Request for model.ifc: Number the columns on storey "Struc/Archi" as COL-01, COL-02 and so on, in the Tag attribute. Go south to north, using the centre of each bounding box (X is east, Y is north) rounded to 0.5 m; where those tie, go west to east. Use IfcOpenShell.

First a look at what the model holds.

```python
import ifcopenshell
import ifcopenshell.util.element
import ifcopenshell.util.placement

model = ifcopenshell.open("model.ifc")
print(model.schema)
storey = next(s for s in model.by_type("IfcBuildingStorey") if s.Name == "Struc/Archi")
columns = [e for e in ifcopenshell.util.element.get_decomposition(storey) if e.is_a("IfcColumn")]
for e in sorted(columns, key=lambda e: e.id()):
    origin = ifcopenshell.util.placement.get_local_placement(e.ObjectPlacement)[:3, 3]
    print(e.id(), e.Tag, e.Name, origin.round(2) + 0.0, sep=" | ")
```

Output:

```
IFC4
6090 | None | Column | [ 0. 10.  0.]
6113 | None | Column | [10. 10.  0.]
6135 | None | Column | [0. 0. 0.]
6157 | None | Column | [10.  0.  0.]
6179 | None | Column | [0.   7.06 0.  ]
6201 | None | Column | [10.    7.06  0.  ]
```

```python
import ifcopenshell
import ifcopenshell.geom
import ifcopenshell.util.element
import ifcopenshell.util.shape

model = ifcopenshell.open("model.ifc")
settings = ifcopenshell.geom.settings()
settings.set("use-world-coords", True)


def centre(element):
    shape = ifcopenshell.geom.create_shape(settings, element)
    return ifcopenshell.util.shape.get_bbox_centroid(shape.geometry)


storey = next(s for s in model.by_type("IfcBuildingStorey") if s.Name == "Struc/Archi")
columns = [e for e in ifcopenshell.util.element.get_decomposition(storey) if e.is_a("IfcColumn")]

# Insertion points can sit at a corner or the storey origin, so sort by the geometry (in metres).
centres = {e: centre(e) for e in columns}
columns.sort(key=lambda e: (round(centres[e][1] / 0.5), centres[e][0]))

for i, e in enumerate(columns, start=1):
    number = f"COL-{i:02d}"
    e.Tag = number
    print(e.id(), number)

model.write("model_edited.ifc")
```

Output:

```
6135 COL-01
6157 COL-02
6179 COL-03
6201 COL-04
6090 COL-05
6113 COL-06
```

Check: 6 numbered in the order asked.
